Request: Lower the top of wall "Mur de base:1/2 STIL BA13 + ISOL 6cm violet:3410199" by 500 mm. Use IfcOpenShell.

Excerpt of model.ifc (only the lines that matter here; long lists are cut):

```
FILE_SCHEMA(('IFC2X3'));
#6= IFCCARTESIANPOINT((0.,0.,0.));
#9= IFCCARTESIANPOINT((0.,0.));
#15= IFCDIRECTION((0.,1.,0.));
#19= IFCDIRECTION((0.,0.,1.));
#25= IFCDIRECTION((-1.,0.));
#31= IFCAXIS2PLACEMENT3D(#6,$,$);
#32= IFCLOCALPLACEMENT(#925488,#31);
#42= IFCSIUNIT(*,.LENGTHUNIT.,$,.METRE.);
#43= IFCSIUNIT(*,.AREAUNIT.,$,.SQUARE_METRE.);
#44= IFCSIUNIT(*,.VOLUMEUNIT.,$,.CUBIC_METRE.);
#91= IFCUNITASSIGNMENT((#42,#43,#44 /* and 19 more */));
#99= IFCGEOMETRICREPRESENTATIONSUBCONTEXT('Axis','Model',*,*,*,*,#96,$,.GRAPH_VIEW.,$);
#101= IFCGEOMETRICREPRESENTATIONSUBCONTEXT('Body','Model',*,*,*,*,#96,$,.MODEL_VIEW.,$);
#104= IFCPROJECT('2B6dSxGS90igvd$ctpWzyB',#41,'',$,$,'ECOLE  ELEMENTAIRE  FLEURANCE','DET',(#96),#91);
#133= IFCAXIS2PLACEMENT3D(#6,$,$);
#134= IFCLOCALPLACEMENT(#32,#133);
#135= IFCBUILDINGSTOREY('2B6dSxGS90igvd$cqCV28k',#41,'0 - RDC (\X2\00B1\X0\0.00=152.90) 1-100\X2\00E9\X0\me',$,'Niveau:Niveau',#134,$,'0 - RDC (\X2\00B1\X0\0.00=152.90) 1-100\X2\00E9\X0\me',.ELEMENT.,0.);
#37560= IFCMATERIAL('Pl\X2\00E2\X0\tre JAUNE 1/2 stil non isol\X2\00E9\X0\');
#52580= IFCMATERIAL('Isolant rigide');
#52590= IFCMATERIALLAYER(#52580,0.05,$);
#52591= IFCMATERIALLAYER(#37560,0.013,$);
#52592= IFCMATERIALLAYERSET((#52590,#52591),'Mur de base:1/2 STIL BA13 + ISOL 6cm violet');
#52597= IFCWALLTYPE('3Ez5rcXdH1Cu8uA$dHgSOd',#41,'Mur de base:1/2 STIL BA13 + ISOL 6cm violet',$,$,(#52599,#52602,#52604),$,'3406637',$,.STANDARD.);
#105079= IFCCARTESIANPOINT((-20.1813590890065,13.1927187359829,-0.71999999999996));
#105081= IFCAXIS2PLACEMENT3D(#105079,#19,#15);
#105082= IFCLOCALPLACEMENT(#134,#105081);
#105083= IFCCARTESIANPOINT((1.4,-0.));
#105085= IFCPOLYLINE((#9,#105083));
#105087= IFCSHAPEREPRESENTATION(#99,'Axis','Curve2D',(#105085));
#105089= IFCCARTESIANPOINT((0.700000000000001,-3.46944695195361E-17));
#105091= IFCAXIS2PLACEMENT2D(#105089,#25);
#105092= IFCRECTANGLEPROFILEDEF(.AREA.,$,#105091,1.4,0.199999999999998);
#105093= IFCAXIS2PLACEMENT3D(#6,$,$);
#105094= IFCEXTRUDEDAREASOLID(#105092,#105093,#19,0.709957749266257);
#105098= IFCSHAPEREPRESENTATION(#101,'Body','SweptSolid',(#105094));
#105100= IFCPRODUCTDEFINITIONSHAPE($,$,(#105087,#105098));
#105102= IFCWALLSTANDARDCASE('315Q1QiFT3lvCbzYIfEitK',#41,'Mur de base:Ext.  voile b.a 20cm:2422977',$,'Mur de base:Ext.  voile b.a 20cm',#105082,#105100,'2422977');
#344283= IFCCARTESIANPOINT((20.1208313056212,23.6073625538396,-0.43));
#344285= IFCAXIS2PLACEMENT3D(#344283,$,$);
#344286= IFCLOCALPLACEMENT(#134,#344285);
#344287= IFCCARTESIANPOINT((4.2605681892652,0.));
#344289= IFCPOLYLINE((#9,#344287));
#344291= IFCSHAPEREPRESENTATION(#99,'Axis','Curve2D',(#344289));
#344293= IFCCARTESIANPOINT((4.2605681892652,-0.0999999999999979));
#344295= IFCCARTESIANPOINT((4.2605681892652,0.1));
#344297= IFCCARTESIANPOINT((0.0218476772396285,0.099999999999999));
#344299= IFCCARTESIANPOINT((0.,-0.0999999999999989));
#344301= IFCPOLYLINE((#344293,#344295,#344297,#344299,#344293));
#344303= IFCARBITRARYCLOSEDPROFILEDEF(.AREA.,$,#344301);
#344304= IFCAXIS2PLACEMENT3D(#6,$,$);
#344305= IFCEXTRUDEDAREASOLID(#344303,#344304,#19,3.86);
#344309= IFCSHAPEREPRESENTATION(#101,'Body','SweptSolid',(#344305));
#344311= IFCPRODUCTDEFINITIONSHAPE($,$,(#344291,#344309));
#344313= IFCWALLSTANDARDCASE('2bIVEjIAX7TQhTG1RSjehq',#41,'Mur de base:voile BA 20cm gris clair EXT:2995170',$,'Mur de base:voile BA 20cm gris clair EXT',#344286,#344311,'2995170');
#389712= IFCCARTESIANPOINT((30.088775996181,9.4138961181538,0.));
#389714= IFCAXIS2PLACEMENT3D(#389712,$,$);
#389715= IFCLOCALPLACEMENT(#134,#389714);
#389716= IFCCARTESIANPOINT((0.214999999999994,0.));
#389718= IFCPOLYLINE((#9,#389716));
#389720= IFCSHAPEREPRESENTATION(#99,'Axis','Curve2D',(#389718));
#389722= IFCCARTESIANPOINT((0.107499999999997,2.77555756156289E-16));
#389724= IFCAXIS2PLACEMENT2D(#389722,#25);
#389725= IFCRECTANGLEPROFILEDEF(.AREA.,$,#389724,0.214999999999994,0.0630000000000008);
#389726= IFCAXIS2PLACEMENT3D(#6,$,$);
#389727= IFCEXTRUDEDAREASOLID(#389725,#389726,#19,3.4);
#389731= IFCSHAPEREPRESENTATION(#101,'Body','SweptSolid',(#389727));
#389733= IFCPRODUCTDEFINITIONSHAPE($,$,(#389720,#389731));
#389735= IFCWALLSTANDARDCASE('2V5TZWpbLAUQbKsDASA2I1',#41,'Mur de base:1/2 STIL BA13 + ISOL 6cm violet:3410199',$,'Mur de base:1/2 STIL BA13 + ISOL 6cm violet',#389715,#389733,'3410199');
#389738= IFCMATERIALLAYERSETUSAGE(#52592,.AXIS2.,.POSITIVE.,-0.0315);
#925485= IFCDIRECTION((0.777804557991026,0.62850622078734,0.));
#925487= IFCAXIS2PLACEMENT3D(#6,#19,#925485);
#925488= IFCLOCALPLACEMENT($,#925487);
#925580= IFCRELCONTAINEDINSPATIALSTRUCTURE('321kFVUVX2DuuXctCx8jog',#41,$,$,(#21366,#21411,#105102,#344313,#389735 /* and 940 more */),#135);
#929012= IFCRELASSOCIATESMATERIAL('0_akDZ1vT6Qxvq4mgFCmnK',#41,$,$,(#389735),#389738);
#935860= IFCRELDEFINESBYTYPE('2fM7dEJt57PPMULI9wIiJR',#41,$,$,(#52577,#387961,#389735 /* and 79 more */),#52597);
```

```python
import ifcopenshell
import ifcopenshell.geom
import ifcopenshell.util.representation
import ifcopenshell.util.shape
import ifcopenshell.util.unit

model = ifcopenshell.open("model.ifc")
unit_scale = ifcopenshell.util.unit.calculate_unit_scale(model)
settings = ifcopenshell.geom.settings()


def volume(element):
    """Net volume in cubic metres, openings subtracted."""
    shape = ifcopenshell.geom.create_shape(settings, element)
    return ifcopenshell.util.shape.get_volume(shape.geometry)


wall = model.by_guid("2V5TZWpbLAUQbKsDASA2I1")
before = volume(wall)

body = ifcopenshell.util.representation.get_representation(wall, "Model", "Body")
solid = body.Items[0]
old_height = solid.Depth
solid.Depth -= 0.5 / unit_scale
after = volume(wall)

print(f"height {old_height:g} -> {solid.Depth:g}, volume {before:.3f} -> {after:.3f} m3")

model.write("model_rev.ifc")
```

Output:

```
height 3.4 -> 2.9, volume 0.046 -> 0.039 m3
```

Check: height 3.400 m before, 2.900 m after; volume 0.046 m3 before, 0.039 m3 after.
